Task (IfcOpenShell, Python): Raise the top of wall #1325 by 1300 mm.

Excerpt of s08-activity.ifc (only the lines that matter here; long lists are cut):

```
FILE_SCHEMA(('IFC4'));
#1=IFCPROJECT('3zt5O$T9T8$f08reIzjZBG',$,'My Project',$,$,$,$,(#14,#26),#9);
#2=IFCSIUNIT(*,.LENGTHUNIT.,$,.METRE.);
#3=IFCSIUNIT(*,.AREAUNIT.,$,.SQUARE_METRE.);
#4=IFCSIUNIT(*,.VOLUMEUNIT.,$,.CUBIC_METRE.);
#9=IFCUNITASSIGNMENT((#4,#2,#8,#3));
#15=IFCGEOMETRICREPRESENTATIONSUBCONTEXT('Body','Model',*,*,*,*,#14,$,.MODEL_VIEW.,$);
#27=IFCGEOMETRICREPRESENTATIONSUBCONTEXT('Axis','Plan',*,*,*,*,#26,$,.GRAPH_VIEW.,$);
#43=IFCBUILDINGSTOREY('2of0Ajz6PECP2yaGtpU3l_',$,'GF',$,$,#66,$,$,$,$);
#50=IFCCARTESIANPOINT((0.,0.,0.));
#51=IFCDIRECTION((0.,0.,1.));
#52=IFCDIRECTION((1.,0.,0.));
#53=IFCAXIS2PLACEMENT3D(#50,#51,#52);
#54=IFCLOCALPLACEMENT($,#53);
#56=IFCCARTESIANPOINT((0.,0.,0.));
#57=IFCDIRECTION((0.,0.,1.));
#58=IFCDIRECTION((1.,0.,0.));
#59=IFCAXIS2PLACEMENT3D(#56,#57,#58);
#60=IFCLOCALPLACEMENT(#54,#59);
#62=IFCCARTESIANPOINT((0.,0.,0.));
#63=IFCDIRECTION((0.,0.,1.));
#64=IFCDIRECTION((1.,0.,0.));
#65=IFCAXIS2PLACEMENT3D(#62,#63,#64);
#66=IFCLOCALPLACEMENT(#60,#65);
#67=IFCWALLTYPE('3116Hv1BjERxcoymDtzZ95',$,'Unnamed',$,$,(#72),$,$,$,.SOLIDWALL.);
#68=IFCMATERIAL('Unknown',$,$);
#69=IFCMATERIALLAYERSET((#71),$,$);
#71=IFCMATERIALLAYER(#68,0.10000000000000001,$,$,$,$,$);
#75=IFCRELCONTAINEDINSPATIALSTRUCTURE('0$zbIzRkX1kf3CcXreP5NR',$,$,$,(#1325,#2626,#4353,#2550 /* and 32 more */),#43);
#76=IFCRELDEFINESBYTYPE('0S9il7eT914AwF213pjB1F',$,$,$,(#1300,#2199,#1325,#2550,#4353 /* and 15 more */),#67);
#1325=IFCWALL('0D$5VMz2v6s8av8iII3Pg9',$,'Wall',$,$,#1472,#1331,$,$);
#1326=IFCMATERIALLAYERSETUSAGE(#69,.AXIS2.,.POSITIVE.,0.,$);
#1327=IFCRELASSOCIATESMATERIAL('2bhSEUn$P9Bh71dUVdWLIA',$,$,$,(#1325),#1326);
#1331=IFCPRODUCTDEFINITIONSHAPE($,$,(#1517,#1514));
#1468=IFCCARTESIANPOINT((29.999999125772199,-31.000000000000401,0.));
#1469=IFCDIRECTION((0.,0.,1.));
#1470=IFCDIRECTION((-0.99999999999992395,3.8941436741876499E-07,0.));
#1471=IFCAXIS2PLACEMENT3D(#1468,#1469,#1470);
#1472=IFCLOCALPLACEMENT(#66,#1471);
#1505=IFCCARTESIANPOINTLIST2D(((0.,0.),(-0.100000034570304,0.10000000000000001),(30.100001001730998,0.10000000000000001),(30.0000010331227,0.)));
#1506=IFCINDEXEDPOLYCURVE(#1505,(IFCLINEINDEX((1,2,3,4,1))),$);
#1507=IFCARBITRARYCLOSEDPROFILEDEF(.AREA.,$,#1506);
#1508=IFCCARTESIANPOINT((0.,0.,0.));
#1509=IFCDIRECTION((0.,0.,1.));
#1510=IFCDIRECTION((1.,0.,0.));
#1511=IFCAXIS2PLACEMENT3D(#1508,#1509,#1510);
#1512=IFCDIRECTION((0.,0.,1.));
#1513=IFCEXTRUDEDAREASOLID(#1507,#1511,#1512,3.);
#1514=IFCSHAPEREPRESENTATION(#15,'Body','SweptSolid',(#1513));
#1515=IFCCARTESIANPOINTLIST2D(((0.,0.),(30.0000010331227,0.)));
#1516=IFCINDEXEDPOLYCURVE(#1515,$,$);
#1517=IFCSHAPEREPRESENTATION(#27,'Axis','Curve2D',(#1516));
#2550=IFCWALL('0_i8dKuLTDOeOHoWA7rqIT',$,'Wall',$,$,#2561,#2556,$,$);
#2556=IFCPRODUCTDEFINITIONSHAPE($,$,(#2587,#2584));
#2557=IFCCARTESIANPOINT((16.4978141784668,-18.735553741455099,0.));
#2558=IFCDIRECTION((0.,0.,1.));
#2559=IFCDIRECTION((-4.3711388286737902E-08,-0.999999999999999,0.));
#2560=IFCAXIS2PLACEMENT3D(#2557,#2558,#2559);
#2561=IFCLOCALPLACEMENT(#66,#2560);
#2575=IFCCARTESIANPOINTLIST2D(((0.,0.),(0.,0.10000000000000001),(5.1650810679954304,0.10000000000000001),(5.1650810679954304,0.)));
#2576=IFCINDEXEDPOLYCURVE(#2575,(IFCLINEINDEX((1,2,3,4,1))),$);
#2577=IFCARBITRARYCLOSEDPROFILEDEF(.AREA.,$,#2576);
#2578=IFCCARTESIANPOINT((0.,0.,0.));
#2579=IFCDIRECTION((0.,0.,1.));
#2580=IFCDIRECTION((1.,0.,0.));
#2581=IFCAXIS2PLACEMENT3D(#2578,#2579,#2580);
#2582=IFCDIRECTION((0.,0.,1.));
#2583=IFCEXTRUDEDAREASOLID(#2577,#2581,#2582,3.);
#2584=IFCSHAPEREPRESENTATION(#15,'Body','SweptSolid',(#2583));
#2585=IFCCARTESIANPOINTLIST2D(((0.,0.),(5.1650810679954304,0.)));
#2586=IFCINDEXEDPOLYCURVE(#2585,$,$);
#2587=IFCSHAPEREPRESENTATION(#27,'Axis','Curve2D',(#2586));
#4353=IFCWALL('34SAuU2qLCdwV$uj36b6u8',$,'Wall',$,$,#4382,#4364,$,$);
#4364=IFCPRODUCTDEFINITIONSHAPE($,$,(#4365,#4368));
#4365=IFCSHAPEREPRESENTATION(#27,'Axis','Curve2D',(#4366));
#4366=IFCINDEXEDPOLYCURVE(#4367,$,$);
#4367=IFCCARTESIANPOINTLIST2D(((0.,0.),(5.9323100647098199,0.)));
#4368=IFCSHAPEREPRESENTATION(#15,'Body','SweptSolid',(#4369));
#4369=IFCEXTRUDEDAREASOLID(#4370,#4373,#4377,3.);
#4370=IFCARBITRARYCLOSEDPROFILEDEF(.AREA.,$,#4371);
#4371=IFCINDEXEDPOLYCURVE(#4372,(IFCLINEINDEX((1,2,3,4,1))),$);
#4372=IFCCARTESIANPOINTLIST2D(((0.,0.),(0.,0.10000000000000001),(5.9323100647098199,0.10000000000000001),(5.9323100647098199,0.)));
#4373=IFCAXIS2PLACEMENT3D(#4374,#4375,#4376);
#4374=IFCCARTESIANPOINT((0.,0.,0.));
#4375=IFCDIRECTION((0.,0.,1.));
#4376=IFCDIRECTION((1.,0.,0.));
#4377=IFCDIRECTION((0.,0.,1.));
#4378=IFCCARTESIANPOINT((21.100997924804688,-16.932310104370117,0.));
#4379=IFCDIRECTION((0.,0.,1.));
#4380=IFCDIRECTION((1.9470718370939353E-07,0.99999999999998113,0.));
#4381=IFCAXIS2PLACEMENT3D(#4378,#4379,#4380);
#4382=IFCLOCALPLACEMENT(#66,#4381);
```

```python
import ifcopenshell
import ifcopenshell.geom
import ifcopenshell.util.representation
import ifcopenshell.util.shape
import ifcopenshell.util.unit

model = ifcopenshell.open("s08-activity.ifc")
unit_scale = ifcopenshell.util.unit.calculate_unit_scale(model)
settings = ifcopenshell.geom.settings()


def volume(element):
    """Net volume in cubic metres, openings subtracted."""
    shape = ifcopenshell.geom.create_shape(settings, element)
    return ifcopenshell.util.shape.get_volume(shape.geometry)


wall = model.by_id(1325)
before = volume(wall)

body = ifcopenshell.util.representation.get_representation(wall, "Model", "Body")
solid = body.Items[0]
old_height = solid.Depth
solid.Depth += 1.3 / unit_scale
after = volume(wall)

print(f"height {old_height:g} -> {solid.Depth:g}, volume {before:.3f} -> {after:.3f} m3")

model.write("s08-activity_v2.ifc")
```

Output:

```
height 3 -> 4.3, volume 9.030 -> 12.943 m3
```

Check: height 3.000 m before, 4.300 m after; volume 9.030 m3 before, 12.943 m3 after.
